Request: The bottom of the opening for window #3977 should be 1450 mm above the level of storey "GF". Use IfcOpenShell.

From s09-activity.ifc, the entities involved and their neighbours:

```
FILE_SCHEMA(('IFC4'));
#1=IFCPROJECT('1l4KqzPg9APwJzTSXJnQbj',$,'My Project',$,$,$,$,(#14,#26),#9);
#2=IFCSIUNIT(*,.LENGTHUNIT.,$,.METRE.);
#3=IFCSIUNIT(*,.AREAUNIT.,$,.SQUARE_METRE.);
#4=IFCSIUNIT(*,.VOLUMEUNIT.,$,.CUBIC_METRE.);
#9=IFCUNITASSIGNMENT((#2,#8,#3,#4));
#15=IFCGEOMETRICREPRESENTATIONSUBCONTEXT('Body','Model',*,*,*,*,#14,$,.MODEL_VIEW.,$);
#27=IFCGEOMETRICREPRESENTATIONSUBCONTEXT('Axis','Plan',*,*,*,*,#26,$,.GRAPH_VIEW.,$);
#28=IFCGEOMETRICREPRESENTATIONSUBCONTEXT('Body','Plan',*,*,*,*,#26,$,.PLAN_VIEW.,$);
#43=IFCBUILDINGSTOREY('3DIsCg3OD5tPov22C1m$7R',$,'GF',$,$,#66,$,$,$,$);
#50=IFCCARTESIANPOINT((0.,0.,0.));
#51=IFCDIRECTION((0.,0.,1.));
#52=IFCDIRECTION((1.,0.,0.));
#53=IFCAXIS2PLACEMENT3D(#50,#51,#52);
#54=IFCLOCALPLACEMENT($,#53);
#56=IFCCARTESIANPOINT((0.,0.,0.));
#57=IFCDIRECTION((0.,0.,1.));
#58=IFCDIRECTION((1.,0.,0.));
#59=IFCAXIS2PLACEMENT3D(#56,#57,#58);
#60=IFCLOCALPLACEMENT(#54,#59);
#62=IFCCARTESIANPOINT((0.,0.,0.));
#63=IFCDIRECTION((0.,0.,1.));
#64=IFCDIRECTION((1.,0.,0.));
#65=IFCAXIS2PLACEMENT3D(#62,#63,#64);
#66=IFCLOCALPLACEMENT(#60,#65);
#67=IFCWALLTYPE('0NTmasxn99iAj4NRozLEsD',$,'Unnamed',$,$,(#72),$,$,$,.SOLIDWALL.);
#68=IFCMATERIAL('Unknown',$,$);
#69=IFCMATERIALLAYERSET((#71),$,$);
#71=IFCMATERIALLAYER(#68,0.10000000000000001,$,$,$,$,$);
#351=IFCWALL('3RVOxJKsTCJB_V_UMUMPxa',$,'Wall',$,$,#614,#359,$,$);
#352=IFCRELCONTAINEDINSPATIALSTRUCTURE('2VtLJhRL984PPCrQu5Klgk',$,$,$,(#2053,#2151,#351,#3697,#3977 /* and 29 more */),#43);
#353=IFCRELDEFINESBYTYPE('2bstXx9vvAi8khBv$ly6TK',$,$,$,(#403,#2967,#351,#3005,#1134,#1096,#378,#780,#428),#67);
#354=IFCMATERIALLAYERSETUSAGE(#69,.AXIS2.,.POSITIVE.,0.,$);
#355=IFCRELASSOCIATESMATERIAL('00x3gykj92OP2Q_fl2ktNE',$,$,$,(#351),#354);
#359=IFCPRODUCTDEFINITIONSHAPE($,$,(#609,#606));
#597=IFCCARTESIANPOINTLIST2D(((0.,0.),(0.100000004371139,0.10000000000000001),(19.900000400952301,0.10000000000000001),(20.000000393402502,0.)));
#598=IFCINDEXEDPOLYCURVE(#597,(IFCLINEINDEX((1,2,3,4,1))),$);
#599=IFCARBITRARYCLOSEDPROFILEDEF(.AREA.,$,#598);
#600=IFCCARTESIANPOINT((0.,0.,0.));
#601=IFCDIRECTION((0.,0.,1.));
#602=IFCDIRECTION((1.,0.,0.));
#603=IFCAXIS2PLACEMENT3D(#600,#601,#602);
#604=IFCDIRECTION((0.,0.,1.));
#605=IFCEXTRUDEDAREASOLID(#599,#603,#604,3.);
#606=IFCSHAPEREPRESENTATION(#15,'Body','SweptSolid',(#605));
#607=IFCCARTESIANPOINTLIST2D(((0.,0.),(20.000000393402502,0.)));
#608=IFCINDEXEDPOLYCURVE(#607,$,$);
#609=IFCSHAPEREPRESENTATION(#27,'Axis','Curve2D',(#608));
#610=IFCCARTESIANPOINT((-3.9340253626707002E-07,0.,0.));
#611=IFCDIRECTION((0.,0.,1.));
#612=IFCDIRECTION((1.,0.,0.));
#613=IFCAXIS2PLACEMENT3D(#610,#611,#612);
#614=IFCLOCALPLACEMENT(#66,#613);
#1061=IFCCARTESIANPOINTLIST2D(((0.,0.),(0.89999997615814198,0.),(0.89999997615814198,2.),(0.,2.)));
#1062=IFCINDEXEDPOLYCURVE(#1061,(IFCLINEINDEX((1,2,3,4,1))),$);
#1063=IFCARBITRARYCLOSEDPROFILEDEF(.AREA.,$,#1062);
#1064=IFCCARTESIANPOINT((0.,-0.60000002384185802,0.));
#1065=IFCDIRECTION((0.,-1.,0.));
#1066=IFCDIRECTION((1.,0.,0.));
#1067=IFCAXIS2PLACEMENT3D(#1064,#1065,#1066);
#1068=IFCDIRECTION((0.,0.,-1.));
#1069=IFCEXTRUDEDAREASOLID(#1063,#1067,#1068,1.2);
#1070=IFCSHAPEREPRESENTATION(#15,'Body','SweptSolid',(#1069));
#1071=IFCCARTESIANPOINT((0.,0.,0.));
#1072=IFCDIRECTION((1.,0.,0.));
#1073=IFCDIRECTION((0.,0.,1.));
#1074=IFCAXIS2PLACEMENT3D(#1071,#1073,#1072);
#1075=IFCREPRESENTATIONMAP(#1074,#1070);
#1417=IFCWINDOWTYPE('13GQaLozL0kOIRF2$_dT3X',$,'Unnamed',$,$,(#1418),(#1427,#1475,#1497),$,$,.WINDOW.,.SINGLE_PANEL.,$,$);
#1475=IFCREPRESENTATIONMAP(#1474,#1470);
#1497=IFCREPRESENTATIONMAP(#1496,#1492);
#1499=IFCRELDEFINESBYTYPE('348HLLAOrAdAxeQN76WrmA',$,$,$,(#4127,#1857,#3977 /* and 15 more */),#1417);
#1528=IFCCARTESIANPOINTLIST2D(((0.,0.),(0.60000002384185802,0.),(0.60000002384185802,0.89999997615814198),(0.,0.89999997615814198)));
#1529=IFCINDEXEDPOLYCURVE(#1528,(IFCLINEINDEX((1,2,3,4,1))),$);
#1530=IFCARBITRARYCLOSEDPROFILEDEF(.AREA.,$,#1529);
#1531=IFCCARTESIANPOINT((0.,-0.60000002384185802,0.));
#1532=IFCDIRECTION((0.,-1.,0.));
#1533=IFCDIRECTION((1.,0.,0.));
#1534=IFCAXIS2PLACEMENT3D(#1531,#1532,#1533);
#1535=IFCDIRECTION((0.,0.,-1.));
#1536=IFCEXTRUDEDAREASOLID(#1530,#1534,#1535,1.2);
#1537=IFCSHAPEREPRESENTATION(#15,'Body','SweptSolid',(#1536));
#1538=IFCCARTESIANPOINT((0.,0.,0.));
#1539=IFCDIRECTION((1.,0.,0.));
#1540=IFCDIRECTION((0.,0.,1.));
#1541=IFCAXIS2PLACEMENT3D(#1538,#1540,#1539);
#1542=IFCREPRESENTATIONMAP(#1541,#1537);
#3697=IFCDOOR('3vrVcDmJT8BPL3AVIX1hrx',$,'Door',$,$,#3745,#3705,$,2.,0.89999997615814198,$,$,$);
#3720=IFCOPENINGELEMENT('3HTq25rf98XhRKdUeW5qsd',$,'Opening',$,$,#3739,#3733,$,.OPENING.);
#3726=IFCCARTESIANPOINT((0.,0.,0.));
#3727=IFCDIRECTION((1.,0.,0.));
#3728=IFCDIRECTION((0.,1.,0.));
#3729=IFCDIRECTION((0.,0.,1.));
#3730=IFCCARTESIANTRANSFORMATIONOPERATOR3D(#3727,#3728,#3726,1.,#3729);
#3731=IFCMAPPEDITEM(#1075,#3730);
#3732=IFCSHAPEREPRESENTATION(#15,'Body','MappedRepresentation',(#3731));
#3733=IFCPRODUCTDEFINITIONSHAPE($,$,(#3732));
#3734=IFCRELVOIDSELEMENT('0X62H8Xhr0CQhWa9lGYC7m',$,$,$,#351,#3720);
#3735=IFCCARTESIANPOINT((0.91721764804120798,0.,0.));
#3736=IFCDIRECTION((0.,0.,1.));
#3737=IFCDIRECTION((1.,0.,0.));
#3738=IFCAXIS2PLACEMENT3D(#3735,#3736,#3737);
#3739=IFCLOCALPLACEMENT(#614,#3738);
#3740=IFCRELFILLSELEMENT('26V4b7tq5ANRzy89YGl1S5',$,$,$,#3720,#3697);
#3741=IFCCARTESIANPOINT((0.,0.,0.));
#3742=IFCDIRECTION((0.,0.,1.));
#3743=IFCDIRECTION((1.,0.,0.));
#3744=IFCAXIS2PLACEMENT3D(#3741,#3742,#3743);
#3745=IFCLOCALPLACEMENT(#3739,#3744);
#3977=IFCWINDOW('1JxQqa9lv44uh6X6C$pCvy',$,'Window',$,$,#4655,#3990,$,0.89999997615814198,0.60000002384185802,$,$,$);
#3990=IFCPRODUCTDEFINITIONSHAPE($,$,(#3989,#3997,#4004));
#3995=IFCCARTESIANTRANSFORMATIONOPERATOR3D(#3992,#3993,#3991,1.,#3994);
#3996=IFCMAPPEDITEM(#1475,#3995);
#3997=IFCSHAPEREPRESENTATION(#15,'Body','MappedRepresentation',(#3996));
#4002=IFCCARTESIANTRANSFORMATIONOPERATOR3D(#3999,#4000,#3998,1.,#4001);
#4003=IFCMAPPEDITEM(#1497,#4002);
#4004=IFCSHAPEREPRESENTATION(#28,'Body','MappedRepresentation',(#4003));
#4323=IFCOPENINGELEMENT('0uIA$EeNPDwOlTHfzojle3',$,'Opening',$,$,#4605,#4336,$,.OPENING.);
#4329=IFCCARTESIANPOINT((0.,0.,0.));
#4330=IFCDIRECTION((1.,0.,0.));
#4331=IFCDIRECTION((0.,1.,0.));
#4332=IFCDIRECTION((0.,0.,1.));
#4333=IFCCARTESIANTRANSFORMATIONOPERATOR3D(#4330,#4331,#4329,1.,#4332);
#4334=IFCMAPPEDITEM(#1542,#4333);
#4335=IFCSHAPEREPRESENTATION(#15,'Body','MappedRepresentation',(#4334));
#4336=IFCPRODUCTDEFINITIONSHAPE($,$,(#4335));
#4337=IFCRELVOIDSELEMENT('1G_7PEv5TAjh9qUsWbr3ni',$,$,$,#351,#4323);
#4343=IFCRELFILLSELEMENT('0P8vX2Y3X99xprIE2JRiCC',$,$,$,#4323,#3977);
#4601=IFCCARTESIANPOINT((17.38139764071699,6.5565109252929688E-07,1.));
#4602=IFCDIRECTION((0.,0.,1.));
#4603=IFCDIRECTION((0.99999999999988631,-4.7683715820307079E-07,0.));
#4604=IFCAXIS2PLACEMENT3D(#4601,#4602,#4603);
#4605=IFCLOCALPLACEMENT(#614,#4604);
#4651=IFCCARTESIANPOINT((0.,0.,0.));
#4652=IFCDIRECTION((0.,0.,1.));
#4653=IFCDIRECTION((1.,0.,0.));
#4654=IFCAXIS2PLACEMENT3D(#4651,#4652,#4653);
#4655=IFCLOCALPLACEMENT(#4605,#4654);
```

```python
import numpy as np
import ifcopenshell
import ifcopenshell.api.geometry
import ifcopenshell.geom
import ifcopenshell.util.element
import ifcopenshell.util.placement
import ifcopenshell.util.shape
import ifcopenshell.util.unit

model = ifcopenshell.open("s09-activity.ifc")
unit_scale = ifcopenshell.util.unit.calculate_unit_scale(model)

window = model.by_guid("1JxQqa9lv44uh6X6C$pCvy")
opening = window.FillsVoids[0].RelatingOpeningElement
storey = ifcopenshell.util.element.get_container(window, ifc_class="IfcBuildingStorey")
level = ifcopenshell.util.placement.get_local_placement(storey.ObjectPlacement)[2, 3]

# The opening's origin need not be at the sill, so measure its lowest point.
shape = ifcopenshell.geom.create_shape(ifcopenshell.geom.settings(), opening)
bottom = ifcopenshell.util.shape.get_shape_bottom_elevation(shape, shape.geometry) / unit_scale
dz = level + 1.45 / unit_scale - bottom

shift = np.array([0.0, 0.0, dz])
# The window is placed relative to its opening, so it follows when the opening moves.
matrix = ifcopenshell.util.placement.get_local_placement(opening.ObjectPlacement)
matrix[:3, 3] += shift
ifcopenshell.api.geometry.edit_object_placement(
    model, product=opening, matrix=matrix, is_si=False, should_transform_children=True
)

print(f"moved by {dz * unit_scale:+.3f} m")

model.write("s09-activity_updated.ifc")
```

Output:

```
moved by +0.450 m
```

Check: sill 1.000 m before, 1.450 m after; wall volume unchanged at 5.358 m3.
